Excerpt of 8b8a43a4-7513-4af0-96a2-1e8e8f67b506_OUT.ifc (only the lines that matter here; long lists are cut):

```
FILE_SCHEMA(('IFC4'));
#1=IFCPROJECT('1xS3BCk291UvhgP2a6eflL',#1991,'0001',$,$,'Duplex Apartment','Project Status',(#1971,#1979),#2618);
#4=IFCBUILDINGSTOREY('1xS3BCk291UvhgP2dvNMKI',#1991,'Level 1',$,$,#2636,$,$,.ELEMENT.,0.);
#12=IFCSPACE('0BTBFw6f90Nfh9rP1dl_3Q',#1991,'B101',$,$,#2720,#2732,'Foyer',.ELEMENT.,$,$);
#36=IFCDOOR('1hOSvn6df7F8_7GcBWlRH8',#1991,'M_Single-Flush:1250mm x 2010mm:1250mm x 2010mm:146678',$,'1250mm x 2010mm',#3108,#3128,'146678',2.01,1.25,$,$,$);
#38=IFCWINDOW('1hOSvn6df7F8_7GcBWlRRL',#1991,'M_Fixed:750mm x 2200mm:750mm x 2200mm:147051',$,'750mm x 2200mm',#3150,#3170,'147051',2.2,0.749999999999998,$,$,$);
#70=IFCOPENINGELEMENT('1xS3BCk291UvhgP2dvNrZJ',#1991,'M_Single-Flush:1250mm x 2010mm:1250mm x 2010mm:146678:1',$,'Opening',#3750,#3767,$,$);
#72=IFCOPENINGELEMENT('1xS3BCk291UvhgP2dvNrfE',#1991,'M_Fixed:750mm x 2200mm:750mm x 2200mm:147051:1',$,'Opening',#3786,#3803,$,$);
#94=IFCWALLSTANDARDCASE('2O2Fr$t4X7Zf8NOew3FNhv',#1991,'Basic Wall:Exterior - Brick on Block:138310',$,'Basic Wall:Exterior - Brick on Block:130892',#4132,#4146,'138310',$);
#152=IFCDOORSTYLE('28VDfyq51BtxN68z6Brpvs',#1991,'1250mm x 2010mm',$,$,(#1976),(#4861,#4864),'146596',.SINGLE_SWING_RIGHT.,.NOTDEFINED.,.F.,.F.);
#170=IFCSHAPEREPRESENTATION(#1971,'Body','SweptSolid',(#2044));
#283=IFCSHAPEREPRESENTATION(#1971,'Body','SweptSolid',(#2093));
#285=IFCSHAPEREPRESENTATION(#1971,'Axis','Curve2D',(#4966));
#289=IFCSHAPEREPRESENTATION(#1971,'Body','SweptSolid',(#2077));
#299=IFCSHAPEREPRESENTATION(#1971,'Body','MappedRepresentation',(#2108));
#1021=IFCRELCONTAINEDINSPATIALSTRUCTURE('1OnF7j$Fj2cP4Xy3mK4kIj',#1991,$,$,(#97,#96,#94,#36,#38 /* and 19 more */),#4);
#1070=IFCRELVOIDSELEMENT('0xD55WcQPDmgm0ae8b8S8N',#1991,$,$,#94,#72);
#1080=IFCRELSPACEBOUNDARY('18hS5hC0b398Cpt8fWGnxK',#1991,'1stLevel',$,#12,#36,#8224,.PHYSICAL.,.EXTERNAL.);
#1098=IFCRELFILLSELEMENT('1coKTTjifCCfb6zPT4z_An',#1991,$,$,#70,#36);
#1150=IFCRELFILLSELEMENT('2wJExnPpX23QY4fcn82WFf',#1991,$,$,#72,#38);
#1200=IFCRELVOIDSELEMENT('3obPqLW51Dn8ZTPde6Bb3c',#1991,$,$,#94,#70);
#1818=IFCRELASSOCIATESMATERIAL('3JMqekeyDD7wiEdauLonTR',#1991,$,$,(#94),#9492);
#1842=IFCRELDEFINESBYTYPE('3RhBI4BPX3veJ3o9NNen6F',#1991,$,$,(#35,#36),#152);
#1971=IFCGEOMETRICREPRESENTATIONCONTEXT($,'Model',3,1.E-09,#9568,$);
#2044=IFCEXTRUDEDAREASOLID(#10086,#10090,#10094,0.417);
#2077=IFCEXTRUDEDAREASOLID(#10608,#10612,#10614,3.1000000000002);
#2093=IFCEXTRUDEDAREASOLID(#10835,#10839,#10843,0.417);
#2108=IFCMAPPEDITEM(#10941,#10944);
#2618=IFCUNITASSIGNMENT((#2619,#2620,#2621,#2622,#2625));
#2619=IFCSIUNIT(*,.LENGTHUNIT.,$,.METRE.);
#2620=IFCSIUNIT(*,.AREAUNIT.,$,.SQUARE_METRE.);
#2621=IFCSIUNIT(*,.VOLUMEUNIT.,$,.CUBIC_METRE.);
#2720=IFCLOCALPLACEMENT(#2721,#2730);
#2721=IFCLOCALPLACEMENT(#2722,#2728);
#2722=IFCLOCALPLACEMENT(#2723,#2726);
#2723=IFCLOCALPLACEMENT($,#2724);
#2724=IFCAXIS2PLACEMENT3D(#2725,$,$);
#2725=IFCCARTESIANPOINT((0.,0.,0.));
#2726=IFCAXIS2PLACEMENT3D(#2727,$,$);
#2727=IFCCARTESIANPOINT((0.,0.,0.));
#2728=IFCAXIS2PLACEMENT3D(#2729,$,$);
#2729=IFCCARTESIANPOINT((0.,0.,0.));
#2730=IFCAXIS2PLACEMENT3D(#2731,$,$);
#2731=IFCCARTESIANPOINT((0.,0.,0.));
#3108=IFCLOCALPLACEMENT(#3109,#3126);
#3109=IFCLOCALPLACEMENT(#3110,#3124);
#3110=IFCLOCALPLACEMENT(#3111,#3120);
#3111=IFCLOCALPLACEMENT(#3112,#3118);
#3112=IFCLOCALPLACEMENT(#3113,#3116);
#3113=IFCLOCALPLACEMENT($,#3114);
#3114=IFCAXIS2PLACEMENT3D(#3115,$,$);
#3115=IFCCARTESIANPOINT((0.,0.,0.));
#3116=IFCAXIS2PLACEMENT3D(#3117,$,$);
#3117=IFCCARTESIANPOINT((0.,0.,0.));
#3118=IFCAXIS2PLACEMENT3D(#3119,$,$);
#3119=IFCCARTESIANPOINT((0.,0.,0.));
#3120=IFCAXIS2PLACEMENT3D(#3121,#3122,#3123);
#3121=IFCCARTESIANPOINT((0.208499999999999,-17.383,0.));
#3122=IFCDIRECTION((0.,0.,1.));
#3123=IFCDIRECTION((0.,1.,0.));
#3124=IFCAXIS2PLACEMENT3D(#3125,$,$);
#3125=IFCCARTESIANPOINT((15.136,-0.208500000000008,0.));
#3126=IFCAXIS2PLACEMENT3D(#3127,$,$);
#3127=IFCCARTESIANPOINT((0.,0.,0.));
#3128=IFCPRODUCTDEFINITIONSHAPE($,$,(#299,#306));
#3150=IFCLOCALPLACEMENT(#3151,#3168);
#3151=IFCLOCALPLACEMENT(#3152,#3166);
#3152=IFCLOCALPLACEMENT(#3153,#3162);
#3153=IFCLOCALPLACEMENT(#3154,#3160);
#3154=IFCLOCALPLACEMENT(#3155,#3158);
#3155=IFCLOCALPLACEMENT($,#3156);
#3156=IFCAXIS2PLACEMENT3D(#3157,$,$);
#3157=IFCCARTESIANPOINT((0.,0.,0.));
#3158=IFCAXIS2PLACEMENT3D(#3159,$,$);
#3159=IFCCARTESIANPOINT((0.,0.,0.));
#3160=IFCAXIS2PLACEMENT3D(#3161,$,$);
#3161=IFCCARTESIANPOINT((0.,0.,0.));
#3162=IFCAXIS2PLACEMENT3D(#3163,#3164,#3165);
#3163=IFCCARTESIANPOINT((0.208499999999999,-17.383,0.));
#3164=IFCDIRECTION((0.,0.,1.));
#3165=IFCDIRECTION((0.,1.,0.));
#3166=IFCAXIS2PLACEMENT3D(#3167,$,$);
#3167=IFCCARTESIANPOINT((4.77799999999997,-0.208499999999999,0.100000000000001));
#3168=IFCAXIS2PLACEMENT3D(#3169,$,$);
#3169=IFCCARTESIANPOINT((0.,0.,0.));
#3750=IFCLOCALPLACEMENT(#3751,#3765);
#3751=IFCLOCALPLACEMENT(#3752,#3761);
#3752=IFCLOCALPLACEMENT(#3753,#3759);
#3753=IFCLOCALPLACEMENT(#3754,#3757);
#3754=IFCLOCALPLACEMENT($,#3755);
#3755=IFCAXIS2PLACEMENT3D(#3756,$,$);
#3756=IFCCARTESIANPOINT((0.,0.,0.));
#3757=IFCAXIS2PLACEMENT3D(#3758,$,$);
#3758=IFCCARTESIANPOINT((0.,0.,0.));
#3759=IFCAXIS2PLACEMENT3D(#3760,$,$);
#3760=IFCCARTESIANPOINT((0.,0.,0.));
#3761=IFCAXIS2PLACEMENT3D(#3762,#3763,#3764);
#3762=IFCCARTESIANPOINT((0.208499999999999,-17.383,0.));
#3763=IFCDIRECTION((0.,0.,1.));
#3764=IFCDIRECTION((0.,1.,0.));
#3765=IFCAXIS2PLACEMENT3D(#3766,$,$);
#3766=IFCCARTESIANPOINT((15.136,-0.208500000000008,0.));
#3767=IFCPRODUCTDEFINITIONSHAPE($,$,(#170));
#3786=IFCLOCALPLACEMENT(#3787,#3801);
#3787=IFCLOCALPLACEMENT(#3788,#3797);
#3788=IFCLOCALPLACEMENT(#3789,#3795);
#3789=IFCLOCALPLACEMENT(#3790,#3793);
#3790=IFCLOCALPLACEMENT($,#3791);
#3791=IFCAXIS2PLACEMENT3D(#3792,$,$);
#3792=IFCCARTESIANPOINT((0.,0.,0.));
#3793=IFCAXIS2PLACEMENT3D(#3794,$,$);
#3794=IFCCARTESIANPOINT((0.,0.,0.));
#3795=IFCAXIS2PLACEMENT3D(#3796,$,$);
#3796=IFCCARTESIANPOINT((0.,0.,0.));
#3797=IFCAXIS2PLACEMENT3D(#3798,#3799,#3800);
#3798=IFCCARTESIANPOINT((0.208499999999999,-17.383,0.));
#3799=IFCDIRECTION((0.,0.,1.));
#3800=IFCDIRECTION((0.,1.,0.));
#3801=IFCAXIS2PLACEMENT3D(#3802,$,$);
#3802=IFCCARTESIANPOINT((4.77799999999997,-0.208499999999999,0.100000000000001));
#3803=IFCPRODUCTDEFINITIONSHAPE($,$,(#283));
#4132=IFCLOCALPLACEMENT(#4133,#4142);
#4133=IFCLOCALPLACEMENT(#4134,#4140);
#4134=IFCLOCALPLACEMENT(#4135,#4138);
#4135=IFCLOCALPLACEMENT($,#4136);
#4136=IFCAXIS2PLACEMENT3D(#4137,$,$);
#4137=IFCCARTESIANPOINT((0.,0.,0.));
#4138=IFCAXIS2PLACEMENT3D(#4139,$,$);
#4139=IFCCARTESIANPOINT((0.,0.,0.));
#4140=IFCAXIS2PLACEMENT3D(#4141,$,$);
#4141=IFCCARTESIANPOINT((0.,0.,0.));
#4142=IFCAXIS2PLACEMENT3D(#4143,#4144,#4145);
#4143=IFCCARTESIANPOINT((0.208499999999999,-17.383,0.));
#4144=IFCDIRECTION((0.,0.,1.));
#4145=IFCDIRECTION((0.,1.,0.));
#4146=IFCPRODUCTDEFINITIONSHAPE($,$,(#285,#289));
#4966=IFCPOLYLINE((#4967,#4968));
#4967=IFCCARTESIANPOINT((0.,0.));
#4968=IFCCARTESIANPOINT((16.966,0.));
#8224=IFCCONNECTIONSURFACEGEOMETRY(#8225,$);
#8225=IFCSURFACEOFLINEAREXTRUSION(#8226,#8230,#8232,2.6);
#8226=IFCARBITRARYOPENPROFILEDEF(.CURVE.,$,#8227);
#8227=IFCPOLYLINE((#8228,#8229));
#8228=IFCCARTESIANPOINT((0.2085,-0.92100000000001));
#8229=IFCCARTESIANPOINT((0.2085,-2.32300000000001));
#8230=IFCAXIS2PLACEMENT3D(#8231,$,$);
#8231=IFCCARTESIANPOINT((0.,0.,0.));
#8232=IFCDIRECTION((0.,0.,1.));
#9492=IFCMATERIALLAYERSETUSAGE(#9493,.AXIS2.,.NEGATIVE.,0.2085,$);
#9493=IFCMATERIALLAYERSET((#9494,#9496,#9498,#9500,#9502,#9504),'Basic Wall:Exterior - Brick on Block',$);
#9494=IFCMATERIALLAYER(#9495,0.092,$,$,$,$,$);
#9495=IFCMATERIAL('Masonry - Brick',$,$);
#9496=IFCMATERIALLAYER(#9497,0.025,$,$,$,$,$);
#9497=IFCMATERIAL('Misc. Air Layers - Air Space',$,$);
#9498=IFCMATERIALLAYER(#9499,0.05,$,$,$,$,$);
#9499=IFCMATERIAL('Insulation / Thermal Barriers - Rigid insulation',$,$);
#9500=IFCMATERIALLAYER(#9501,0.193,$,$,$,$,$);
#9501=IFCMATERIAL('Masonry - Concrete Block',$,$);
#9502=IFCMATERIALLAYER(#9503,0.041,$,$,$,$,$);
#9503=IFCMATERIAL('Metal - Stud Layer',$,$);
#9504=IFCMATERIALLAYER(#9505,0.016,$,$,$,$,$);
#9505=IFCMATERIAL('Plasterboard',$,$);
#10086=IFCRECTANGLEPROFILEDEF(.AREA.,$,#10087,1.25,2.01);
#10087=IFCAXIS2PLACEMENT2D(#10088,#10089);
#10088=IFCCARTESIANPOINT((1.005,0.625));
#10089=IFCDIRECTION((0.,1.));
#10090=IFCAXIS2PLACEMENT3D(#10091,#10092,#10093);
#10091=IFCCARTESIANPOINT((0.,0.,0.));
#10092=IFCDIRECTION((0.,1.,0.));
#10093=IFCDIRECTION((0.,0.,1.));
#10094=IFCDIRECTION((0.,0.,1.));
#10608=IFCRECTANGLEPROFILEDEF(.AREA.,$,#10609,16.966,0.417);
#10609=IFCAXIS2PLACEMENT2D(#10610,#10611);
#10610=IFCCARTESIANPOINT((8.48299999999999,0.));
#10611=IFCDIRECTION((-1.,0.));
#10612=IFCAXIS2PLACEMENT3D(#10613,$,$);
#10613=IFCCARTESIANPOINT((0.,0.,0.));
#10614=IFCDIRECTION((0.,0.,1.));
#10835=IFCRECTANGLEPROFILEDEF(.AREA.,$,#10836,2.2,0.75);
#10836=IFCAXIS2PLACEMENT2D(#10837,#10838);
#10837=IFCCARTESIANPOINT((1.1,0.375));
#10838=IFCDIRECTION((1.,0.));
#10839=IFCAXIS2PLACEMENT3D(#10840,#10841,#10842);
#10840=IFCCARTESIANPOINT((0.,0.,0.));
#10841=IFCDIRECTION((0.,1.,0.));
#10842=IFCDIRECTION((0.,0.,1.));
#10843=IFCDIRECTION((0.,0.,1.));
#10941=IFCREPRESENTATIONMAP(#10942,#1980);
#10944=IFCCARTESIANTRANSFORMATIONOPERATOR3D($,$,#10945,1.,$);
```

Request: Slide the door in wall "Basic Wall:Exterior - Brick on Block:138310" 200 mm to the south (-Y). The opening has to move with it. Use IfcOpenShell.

```python
import numpy as np
import ifcopenshell
import ifcopenshell.api.geometry
import ifcopenshell.util.placement

model = ifcopenshell.open("8b8a43a4-7513-4af0-96a2-1e8e8f67b506_OUT.ifc")

door = model.by_guid("1hOSvn6df7F8_7GcBWlRH8")
opening = door.FillsVoids[0].RelatingOpeningElement
wall = opening.VoidsElements[0].RelatingBuildingElement

wall_matrix = ifcopenshell.util.placement.get_local_placement(wall.ObjectPlacement)
shift = wall_matrix[:3, 0] * -0.2
before = ifcopenshell.util.placement.get_local_placement(door.ObjectPlacement)[:3, 3].copy()

# The door is not placed relative to its opening, so move both.
for product in (opening, door):
    matrix = ifcopenshell.util.placement.get_local_placement(product.ObjectPlacement)
    matrix[:3, 3] += shift
    ifcopenshell.api.geometry.edit_object_placement(model, product=product, matrix=matrix, is_si=False)

# Space boundary surfaces are stored in each space's coordinates; move them too.
for rel in door.ProvidesBoundaries:
    if not rel.ConnectionGeometry:
        continue
    surface = rel.ConnectionGeometry.SurfaceOnRelatingElement
    space_matrix = ifcopenshell.util.placement.get_local_placement(rel.RelatingSpace.ObjectPlacement)
    point = np.array(surface.Position.Location.Coordinates) + space_matrix[:3, :3].T @ shift
    surface.Position = model.createIfcAxis2Placement3D(
        model.createIfcCartesianPoint(point.tolist()), surface.Position.Axis, surface.Position.RefDirection
    )

after = ifcopenshell.util.placement.get_local_placement(door.ObjectPlacement)[:3, 3]
print("door moved by", (after - before).round(3) + 0.0)

model.write("8b8a43a4-7513-4af0-96a2-1e8e8f67b506_OUT_v2.ifc")
```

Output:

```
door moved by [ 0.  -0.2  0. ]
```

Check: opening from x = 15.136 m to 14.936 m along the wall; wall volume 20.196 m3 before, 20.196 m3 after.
